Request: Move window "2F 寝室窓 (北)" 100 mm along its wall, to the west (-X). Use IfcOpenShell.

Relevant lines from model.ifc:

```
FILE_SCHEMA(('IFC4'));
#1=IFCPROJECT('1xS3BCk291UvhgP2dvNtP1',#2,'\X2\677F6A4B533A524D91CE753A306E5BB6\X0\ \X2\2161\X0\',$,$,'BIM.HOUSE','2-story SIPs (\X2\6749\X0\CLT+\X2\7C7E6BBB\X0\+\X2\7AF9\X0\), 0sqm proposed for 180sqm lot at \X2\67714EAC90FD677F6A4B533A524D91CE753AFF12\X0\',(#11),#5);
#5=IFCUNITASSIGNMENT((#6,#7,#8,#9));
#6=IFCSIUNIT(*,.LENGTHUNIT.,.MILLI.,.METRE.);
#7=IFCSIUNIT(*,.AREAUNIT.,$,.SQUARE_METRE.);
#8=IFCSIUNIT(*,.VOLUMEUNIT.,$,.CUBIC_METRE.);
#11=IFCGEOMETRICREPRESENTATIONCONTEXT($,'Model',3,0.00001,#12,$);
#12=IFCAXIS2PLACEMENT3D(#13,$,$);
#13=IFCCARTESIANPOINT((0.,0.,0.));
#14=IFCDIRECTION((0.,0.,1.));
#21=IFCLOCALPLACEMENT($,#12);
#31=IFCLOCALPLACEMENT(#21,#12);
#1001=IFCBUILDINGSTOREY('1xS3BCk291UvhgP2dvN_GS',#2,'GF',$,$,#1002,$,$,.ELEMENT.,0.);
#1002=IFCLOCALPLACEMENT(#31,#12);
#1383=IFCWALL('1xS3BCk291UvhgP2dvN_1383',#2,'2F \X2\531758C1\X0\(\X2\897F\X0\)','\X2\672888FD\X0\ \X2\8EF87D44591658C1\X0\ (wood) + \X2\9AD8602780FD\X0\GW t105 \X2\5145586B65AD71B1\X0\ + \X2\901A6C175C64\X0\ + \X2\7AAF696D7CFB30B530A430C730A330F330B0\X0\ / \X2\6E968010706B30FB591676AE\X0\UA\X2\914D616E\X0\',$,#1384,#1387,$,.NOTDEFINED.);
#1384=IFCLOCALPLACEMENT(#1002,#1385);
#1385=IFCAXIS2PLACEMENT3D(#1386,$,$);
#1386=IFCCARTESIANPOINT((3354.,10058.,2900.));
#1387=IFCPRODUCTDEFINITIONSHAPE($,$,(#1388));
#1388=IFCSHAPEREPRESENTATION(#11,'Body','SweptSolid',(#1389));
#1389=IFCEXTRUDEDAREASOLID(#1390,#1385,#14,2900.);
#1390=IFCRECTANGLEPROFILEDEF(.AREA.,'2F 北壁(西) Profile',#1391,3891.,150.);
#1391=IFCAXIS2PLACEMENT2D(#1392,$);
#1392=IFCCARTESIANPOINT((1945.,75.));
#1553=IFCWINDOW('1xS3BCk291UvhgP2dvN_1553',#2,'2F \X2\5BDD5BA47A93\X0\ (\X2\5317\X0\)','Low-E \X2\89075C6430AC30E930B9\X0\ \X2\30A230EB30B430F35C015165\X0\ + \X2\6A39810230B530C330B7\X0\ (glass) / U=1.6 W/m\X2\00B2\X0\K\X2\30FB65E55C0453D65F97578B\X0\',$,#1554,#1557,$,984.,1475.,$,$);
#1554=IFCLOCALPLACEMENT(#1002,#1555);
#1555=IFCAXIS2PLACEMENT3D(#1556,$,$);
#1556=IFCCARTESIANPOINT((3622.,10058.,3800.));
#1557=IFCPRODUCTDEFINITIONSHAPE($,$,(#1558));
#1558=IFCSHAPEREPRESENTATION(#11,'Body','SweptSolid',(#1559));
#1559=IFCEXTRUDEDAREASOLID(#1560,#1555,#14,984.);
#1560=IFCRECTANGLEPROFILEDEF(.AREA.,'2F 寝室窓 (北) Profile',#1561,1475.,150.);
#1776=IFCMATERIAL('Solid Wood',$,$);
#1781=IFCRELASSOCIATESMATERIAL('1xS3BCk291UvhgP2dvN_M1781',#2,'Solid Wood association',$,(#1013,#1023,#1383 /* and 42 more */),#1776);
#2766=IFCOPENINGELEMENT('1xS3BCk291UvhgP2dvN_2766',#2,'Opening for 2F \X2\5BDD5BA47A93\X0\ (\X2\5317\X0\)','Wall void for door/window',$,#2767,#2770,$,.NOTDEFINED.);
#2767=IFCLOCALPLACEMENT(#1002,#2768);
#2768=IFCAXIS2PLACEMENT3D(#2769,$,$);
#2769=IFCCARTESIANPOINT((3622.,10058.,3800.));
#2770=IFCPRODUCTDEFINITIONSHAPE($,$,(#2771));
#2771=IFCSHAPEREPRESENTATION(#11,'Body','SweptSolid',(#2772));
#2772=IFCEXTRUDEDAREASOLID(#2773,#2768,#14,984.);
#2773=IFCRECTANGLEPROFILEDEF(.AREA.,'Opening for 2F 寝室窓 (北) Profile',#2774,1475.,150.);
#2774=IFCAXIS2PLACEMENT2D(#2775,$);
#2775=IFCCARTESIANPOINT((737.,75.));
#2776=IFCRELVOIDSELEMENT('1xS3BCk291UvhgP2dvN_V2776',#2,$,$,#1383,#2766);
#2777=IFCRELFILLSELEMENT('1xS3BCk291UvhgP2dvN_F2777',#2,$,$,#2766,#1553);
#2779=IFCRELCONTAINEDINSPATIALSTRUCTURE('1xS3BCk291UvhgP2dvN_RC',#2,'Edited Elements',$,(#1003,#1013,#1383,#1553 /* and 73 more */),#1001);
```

```python
import ifcopenshell
import ifcopenshell.api.geometry
import ifcopenshell.util.placement

model = ifcopenshell.open("model.ifc")

window = model.by_guid("1xS3BCk291UvhgP2dvN_1553")
opening = window.FillsVoids[0].RelatingOpeningElement
wall = opening.VoidsElements[0].RelatingBuildingElement

wall_matrix = ifcopenshell.util.placement.get_local_placement(wall.ObjectPlacement)
shift = wall_matrix[:3, 0] * -100.0
before = ifcopenshell.util.placement.get_local_placement(window.ObjectPlacement)[:3, 3].copy()

# The window is not placed relative to its opening, so move both.
for product in (opening, window):
    matrix = ifcopenshell.util.placement.get_local_placement(product.ObjectPlacement)
    matrix[:3, 3] += shift
    ifcopenshell.api.geometry.edit_object_placement(model, product=product, matrix=matrix, is_si=False)

after = ifcopenshell.util.placement.get_local_placement(window.ObjectPlacement)[:3, 3]
print("window moved by", (after - before).round(3) + 0.0)

model.write("model_rev.ifc")
```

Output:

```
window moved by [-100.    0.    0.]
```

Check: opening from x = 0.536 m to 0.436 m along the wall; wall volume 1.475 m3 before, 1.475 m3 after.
